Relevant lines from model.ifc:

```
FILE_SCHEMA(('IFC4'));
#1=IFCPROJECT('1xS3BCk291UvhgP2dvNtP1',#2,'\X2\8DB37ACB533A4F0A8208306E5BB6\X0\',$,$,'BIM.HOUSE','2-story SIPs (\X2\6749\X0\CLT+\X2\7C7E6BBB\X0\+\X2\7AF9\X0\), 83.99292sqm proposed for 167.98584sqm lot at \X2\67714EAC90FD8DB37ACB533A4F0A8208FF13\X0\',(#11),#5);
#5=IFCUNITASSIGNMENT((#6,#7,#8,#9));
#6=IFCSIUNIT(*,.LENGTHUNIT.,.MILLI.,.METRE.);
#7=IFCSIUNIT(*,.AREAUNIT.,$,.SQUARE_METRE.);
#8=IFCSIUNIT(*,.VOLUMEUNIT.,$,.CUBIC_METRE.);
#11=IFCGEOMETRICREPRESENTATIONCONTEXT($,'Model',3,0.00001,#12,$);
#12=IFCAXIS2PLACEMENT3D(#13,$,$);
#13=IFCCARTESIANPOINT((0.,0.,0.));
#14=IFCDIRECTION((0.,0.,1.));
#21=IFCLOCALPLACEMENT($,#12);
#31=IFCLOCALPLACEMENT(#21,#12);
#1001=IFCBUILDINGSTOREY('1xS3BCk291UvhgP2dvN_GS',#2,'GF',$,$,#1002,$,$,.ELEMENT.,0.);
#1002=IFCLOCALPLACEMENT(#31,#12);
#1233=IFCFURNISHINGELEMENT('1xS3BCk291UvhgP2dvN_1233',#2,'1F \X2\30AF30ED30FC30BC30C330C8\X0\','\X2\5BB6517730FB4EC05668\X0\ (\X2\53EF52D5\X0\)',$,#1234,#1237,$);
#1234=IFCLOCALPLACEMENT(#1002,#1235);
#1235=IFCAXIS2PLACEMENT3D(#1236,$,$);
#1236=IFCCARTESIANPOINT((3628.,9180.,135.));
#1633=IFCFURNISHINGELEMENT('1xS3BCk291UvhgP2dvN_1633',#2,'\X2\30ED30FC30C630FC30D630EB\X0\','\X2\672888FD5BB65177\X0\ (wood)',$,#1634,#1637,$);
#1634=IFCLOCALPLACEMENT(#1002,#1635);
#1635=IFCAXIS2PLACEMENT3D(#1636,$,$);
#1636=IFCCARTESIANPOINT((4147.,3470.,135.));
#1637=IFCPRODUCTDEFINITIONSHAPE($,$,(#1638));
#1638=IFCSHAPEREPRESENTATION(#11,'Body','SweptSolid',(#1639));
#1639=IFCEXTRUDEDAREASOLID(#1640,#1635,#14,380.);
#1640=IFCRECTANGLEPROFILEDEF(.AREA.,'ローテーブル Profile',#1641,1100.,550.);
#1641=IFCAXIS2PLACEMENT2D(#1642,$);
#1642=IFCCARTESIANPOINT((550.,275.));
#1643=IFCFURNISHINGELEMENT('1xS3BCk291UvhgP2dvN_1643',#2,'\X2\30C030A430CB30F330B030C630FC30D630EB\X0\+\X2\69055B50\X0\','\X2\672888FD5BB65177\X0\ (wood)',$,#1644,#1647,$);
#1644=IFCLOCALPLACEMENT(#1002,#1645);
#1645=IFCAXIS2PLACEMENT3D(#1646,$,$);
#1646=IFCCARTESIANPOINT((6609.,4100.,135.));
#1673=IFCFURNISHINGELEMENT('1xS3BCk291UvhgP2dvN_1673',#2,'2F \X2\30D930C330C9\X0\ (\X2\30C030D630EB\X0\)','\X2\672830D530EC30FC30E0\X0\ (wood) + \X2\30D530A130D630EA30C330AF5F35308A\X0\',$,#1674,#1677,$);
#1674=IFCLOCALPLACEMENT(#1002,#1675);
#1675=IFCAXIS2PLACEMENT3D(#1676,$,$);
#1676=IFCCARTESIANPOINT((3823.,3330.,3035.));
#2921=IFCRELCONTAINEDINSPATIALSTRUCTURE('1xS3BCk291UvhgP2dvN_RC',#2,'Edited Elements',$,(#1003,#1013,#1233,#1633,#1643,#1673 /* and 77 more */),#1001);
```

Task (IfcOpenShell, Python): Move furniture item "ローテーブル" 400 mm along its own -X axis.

```python
import ifcopenshell
import ifcopenshell.api.geometry
import ifcopenshell.util.placement

model = ifcopenshell.open("model.ifc")

item = model.by_guid("1xS3BCk291UvhgP2dvN_1633")
matrix = ifcopenshell.util.placement.get_local_placement(item.ObjectPlacement)
matrix[:3, 3] -= matrix[:3, 0] * 400.0
ifcopenshell.api.geometry.edit_object_placement(model, product=item, matrix=matrix, is_si=False)

print(ifcopenshell.util.placement.get_local_placement(item.ObjectPlacement).round(3) + 0.0)

model.write("model-out.ifc")
```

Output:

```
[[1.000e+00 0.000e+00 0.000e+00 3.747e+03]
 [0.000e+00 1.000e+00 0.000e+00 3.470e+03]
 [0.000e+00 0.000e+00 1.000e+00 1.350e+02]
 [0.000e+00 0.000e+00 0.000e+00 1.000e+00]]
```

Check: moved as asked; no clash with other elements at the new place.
